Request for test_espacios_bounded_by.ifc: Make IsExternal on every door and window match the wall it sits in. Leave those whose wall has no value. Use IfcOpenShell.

First a look at what the model holds.

```python
import ifcopenshell
import ifcopenshell.util.element

model = ifcopenshell.open("test_espacios_bounded_by.ifc")
print(model.schema)
seen = {}
for e in model.by_type("IfcDoor") + model.by_type("IfcWindow"):
    if not e.FillsVoids:
        continue
    host = e.FillsVoids[0].RelatingOpeningElement.VoidsElements[0].RelatingBuildingElement
    own = ifcopenshell.util.element.get_pset(e, f"Pset_{e.is_a()[3:].removesuffix('StandardCase')}Common", "IsExternal")
    wall = ifcopenshell.util.element.get_pset(host, "Pset_WallCommon", "IsExternal")
    seen[e.is_a(), own, wall] = seen.get((e.is_a(), own, wall), 0) + 1
for (cls, own, wall), count in sorted(seen.items(), key=str):
    print(count, cls, "IsExternal:", own, "| host wall:", wall)
```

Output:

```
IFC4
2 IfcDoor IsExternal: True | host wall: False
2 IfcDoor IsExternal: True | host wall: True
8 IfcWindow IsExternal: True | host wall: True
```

```python
import ifcopenshell
import ifcopenshell.api.pset
import ifcopenshell.util.element

model = ifcopenshell.open("test_espacios_bounded_by.ifc")

count = 0
for ifc_class, pset_name in (("IfcDoor", "Pset_DoorCommon"), ("IfcWindow", "Pset_WindowCommon")):
    for e in model.by_type(ifc_class):
        if not e.FillsVoids:
            continue
        host = e.FillsVoids[0].RelatingOpeningElement.VoidsElements[0].RelatingBuildingElement
        external = ifcopenshell.util.element.get_pset(host, "Pset_WallCommon", "IsExternal")
        if external is None or ifcopenshell.util.element.get_pset(e, pset_name, "IsExternal") == external:
            continue
        pset = ifcopenshell.api.pset.add_pset(model, product=e, name=pset_name)
        ifcopenshell.api.pset.edit_pset(model, pset=pset, properties={"IsExternal": external})
        count += 1

print(count, "updated")

model.write("test_espacios_bounded_by_updated.ifc")
```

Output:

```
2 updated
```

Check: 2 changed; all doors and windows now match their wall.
